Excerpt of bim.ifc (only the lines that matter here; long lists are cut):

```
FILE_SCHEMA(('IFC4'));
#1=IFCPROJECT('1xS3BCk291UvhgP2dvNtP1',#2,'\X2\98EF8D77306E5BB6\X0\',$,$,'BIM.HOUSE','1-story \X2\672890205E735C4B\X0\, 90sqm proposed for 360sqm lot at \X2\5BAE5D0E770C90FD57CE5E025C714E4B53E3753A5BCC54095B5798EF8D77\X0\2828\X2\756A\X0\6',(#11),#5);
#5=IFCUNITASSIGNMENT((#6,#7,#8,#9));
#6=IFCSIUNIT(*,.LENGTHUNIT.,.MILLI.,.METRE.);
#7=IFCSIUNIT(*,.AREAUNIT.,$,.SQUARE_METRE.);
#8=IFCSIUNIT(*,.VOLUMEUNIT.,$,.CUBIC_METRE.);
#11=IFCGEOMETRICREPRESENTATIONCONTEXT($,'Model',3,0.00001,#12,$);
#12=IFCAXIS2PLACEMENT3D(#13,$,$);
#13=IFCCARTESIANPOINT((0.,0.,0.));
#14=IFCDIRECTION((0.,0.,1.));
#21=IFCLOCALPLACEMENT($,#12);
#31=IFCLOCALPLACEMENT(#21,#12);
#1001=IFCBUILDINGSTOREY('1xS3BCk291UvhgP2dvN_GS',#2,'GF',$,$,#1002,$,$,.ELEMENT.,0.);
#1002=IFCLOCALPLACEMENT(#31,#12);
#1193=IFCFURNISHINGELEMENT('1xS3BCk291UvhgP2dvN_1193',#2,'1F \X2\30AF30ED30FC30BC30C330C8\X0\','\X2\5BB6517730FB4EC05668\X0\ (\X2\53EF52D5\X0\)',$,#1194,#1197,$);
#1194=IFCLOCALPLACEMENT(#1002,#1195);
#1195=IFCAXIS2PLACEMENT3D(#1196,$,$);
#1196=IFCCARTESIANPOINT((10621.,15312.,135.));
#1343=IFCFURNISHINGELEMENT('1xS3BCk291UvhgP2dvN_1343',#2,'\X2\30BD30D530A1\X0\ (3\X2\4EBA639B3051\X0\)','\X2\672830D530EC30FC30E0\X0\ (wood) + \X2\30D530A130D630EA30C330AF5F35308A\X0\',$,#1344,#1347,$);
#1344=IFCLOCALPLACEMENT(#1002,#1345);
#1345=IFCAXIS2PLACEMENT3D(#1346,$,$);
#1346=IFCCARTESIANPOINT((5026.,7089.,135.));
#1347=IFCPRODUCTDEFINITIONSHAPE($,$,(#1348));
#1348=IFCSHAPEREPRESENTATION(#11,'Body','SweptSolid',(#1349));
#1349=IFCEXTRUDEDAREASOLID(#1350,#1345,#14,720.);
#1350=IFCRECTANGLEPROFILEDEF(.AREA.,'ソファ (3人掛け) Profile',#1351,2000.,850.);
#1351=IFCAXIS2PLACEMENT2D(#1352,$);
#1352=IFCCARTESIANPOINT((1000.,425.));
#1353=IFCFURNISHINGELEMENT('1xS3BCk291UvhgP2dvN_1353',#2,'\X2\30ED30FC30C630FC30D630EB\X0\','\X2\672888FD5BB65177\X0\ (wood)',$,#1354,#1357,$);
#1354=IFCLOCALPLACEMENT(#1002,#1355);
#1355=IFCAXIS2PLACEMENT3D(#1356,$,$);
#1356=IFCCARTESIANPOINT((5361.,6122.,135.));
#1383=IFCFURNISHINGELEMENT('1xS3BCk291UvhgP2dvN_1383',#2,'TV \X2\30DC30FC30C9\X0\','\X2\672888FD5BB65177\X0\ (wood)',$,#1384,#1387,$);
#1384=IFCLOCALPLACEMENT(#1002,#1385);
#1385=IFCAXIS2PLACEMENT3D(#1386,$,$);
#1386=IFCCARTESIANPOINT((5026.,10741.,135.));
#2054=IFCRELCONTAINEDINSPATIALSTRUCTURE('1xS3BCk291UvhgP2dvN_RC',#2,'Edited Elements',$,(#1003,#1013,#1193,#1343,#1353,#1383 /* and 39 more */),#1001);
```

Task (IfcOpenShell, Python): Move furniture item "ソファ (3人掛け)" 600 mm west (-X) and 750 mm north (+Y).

```python
import ifcopenshell
import ifcopenshell.api.geometry
import ifcopenshell.util.placement
import ifcopenshell.util.unit

model = ifcopenshell.open("bim.ifc")
unit_scale = ifcopenshell.util.unit.calculate_unit_scale(model)

item = model.by_guid("1xS3BCk291UvhgP2dvN_1343")
matrix = ifcopenshell.util.placement.get_local_placement(item.ObjectPlacement)
matrix[0, 3] -= 0.6 / unit_scale
matrix[1, 3] += 0.75 / unit_scale
ifcopenshell.api.geometry.edit_object_placement(model, product=item, matrix=matrix, is_si=False)

print(ifcopenshell.util.placement.get_local_placement(item.ObjectPlacement).round(3) + 0.0)

model.write("bim-out.ifc")
```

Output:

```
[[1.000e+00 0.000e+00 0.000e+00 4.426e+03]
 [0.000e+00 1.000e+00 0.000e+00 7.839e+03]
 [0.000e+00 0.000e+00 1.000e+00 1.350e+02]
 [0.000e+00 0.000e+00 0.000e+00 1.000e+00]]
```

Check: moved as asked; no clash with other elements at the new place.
